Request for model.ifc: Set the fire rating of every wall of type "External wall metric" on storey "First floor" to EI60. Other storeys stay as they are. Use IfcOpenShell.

First a look at what the model holds.

```python
import ifcopenshell
import ifcopenshell.util.element

model = ifcopenshell.open("model.ifc")
print(model.schema)
storey = next(s for s in model.by_type("IfcBuildingStorey") if s.Name == "First floor")
walls = [e for e in ifcopenshell.util.element.get_decomposition(storey) if e.is_a("IfcWall")]
seen = {}
for e in walls:
    element_type = ifcopenshell.util.element.get_type(e)
    key = (element_type.Name if element_type != e and element_type else None, ifcopenshell.util.element.get_pset(e, "Pset_WallCommon", "FireRating"))
    seen[key] = seen.get(key, 0) + 1
for (name, value), count in sorted(seen.items(), key=str):
    print(count, "x", name, "|", value)
```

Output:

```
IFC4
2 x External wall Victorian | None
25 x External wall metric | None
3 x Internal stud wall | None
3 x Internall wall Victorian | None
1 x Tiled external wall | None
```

```python
import ifcopenshell
import ifcopenshell.api.pset
import ifcopenshell.util.element

model = ifcopenshell.open("model.ifc")

storey = next(s for s in model.by_type("IfcBuildingStorey") if s.Name == "First floor")
walls = [e for e in ifcopenshell.util.element.get_decomposition(storey) if e.is_a("IfcWall")]

count = 0
for e in walls:
    element_type = ifcopenshell.util.element.get_type(e)
    if element_type in (None, e) or element_type.Name != "External wall metric":
        continue
    # add_pset returns the element's existing set when there is one.
    pset = ifcopenshell.api.pset.add_pset(model, product=e, name="Pset_WallCommon")
    ifcopenshell.api.pset.edit_pset(model, pset=pset, properties={"FireRating": "EI60"})
    count += 1

print(count, "walls updated")

model.write("model-out.ifc")
```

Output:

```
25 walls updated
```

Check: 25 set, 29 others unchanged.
